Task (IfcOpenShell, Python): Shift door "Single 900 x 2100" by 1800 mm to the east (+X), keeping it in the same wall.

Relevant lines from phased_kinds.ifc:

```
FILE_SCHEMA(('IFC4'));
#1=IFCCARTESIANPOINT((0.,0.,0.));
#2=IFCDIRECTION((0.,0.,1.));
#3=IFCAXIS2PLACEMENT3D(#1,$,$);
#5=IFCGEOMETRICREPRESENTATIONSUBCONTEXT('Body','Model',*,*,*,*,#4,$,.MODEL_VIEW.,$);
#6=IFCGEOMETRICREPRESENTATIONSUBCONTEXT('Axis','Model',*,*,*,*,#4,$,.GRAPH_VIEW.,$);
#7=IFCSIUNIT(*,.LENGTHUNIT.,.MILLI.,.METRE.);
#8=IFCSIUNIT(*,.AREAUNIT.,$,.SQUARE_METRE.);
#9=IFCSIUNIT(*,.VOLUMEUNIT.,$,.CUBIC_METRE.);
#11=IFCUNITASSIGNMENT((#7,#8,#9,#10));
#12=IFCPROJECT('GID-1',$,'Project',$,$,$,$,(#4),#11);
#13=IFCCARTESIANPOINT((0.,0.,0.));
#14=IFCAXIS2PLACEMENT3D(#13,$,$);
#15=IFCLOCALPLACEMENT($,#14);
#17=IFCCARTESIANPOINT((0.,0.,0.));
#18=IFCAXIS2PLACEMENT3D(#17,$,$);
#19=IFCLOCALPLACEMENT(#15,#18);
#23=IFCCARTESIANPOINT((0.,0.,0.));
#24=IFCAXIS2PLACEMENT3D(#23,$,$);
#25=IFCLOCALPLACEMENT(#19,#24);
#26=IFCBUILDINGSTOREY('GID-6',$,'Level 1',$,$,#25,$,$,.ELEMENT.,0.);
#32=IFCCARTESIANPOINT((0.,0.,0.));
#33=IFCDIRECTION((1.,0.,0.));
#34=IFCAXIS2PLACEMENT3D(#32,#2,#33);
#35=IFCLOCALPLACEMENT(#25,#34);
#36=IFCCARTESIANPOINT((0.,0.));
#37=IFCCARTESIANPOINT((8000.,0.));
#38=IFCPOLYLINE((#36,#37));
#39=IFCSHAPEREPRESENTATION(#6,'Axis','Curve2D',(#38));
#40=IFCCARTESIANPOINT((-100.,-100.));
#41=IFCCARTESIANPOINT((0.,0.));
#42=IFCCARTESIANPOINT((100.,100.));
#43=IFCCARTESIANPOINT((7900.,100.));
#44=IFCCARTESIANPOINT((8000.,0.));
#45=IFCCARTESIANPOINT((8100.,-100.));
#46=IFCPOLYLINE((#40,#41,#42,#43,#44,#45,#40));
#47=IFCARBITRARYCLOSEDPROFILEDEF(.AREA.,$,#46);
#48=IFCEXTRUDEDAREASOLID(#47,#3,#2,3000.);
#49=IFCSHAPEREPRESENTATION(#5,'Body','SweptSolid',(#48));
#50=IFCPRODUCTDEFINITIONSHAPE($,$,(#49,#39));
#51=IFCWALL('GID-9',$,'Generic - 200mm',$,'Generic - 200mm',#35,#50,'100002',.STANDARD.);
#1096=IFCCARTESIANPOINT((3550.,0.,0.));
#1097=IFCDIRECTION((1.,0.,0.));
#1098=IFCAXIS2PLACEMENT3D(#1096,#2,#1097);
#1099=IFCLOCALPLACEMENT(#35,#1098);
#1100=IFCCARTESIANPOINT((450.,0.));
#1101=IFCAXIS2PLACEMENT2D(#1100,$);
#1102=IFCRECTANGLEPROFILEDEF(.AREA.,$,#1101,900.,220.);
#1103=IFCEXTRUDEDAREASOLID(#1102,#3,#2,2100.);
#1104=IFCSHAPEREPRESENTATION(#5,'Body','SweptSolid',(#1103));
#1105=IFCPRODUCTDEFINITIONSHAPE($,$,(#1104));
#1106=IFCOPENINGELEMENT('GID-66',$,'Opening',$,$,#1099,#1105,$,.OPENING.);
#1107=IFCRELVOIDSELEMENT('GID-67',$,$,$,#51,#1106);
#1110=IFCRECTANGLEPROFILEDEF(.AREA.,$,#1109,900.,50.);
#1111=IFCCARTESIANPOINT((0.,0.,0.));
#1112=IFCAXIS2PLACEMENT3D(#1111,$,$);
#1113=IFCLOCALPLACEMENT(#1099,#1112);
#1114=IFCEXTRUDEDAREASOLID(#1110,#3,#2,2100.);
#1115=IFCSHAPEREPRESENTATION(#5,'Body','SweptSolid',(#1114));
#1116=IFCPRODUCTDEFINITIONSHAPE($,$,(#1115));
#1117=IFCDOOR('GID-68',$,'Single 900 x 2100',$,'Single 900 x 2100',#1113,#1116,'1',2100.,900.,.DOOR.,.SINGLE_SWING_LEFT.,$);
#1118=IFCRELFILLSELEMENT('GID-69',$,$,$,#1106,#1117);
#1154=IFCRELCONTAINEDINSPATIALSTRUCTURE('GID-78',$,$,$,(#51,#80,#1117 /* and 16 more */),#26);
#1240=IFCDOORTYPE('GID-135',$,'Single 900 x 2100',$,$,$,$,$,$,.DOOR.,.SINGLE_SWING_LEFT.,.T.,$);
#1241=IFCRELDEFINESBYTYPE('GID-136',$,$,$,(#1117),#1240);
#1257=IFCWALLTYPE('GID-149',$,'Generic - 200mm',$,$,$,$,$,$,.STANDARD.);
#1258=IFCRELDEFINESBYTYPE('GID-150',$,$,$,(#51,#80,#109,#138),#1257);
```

```python
import ifcopenshell
import ifcopenshell.api.geometry
import ifcopenshell.util.placement

model = ifcopenshell.open("phased_kinds.ifc")

door = model.by_guid("GID-68")
opening = door.FillsVoids[0].RelatingOpeningElement
wall = opening.VoidsElements[0].RelatingBuildingElement

wall_matrix = ifcopenshell.util.placement.get_local_placement(wall.ObjectPlacement)
shift = wall_matrix[:3, 0] * 1800.0
before = ifcopenshell.util.placement.get_local_placement(door.ObjectPlacement)[:3, 3].copy()

# The door is placed relative to its opening, so it follows when the opening moves.
matrix = ifcopenshell.util.placement.get_local_placement(opening.ObjectPlacement)
matrix[:3, 3] += shift
ifcopenshell.api.geometry.edit_object_placement(
    model, product=opening, matrix=matrix, is_si=False, should_transform_children=True
)

after = ifcopenshell.util.placement.get_local_placement(door.ObjectPlacement)[:3, 3]
print("door moved by", (after - before).round(3) + 0.0)

model.write("phased_kinds_updated.ifc")
```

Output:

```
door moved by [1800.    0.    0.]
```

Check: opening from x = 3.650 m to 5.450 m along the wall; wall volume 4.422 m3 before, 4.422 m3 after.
